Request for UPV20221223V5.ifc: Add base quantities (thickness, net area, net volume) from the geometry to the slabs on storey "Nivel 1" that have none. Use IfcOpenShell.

First a look at what the model holds.

```python
import ifcopenshell
import ifcopenshell.util.element
import ifcopenshell.util.unit

model = ifcopenshell.open("UPV20221223V5.ifc")
print(model.schema)
for unit_type in ("LENGTHUNIT", "AREAUNIT", "VOLUMEUNIT"):
    print(unit_type, ifcopenshell.util.unit.calculate_unit_scale(model, unit_type))
storey = next(s for s in model.by_type("IfcBuildingStorey") if s.Name == "Nivel 1")
slabs = [e for e in ifcopenshell.util.element.get_decomposition(storey) if e.is_a("IfcSlab")]
for e in sorted(slabs, key=lambda e: e.id()):
    print(e.id(), e.is_a(), e.Name, list(ifcopenshell.util.element.get_psets(e, qtos_only=True)), sep=" | ")
```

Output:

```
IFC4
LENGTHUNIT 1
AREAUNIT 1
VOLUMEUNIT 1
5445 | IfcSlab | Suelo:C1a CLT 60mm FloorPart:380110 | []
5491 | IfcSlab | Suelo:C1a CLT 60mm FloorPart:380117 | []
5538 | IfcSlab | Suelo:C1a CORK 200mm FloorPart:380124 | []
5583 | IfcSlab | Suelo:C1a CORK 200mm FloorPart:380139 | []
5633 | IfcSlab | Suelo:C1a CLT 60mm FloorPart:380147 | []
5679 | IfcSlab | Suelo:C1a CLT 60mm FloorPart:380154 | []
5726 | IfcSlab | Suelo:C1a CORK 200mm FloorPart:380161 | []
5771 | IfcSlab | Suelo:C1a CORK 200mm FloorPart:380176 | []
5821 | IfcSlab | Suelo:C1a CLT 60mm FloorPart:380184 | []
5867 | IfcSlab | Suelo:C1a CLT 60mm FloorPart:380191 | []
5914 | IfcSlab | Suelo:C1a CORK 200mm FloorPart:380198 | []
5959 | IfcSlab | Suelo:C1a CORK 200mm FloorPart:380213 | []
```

```python
import ifcopenshell
import ifcopenshell.api.pset
import ifcopenshell.geom
import ifcopenshell.util.element
import ifcopenshell.util.shape
import ifcopenshell.util.unit

model = ifcopenshell.open("UPV20221223V5.ifc")
unit_scale = ifcopenshell.util.unit.calculate_unit_scale(model)
area_scale = ifcopenshell.util.unit.calculate_unit_scale(model, "AREAUNIT")
volume_scale = ifcopenshell.util.unit.calculate_unit_scale(model, "VOLUMEUNIT")
settings = ifcopenshell.geom.settings()

storey = next(s for s in model.by_type("IfcBuildingStorey") if s.Name == "Nivel 1")
slabs = [e for e in ifcopenshell.util.element.get_decomposition(storey) if e.is_a("IfcSlab")]

for e in sorted(slabs, key=lambda e: e.id()):
    if ifcopenshell.util.element.get_psets(e, qtos_only=True, should_inherit=False):
        continue
    # Geometry comes back in metres, in the element's own axes.
    shape = ifcopenshell.geom.create_shape(settings, e)
    values = {
        "Width": ifcopenshell.util.shape.get_z(shape.geometry) / unit_scale,
        "NetArea": ifcopenshell.util.shape.get_footprint_area(shape.geometry) / area_scale,
        "NetVolume": ifcopenshell.util.shape.get_volume(shape.geometry) / volume_scale,
    }
    qto = ifcopenshell.api.pset.add_qto(model, product=e, name="Qto_SlabBaseQuantities")
    ifcopenshell.api.pset.edit_qto(model, qto=qto, properties=values)
    print(e.id(), {k: round(v, 3) for k, v in values.items()})

model.write("UPV20221223V5_updated.ifc")
```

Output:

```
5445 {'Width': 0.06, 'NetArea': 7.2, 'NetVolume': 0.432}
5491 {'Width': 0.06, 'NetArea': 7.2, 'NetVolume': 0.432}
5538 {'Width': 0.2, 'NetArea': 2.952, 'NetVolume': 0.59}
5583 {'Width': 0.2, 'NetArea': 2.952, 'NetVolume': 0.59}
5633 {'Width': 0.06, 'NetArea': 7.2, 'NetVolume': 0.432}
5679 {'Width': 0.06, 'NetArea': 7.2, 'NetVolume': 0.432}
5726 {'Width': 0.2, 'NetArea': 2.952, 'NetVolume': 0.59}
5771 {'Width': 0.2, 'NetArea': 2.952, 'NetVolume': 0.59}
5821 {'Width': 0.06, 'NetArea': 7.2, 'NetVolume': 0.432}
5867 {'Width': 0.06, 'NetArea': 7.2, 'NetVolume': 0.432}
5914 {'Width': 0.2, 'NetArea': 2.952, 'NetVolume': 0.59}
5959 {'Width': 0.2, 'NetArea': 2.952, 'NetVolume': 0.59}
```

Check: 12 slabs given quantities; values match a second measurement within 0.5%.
